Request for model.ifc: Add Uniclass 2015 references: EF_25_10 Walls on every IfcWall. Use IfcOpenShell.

First a look at what the model holds.

```python
import ifcopenshell

model = ifcopenshell.open("model.ifc")
print(model.schema)
print("classifications:", [c.Name for c in model.by_type("IfcClassification")])
for ifc_class in ("IfcDoor", "IfcRoof", "IfcStair", "IfcWall", "IfcWindow"):
    print(ifc_class, len(model.by_type(ifc_class)))
```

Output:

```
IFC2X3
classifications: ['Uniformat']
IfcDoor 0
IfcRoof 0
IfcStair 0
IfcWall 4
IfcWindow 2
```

```python
import ifcopenshell
import ifcopenshell.api.classification

model = ifcopenshell.open("model.ifc")

# IFC2X3 requires Source and Edition and has no link from the project to the system.
system = model.create_entity("IfcClassification", Source="NBS", Edition="2015", Name="Uniclass 2015")

codes = {
    "IfcWall": ("EF_25_10", "Walls"),
}
for ifc_class, (code, name) in codes.items():
    products = model.by_type(ifc_class)
    ifcopenshell.api.classification.add_reference(
        model, products=products, classification=system, identification=code, name=name
    )
    print(code, len(products))

model.write("model_updated.ifc")
```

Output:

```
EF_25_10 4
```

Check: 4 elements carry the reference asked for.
